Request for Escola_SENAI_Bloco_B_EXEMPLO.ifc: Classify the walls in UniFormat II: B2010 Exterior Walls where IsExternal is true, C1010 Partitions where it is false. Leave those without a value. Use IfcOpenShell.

First a look at what the model holds.

```python
import ifcopenshell
import ifcopenshell.util.element

model = ifcopenshell.open("Escola_SENAI_Bloco_B_EXEMPLO.ifc")
print(model.schema)
print("classifications:", [c.Name for c in model.by_type("IfcClassification")])
values = [ifcopenshell.util.element.get_pset(e, "Pset_WallCommon", "IsExternal") for e in model.by_type("IfcWall")]
for value in (True, False, None):
    print("IsExternal", value, values.count(value))
```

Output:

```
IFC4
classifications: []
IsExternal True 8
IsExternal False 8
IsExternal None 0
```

```python
import ifcopenshell
import ifcopenshell.api.classification
import ifcopenshell.util.element

model = ifcopenshell.open("Escola_SENAI_Bloco_B_EXEMPLO.ifc")

system = ifcopenshell.api.classification.add_classification(model, classification="UniFormat II")

walls = model.by_type("IfcWall")
external = {e: ifcopenshell.util.element.get_pset(e, "Pset_WallCommon", "IsExternal") for e in walls}
for flag, code, name in ((True, "B2010", "Exterior Walls"), (False, "C1010", "Partitions")):
    products = [e for e in walls if external[e] is flag]
    ifcopenshell.api.classification.add_reference(
        model, products=products, classification=system, identification=code, name=name
    )
    print(code, len(products))

model.write("Escola_SENAI_Bloco_B_EXEMPLO_edited.ifc")
```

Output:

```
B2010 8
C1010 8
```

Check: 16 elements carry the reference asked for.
